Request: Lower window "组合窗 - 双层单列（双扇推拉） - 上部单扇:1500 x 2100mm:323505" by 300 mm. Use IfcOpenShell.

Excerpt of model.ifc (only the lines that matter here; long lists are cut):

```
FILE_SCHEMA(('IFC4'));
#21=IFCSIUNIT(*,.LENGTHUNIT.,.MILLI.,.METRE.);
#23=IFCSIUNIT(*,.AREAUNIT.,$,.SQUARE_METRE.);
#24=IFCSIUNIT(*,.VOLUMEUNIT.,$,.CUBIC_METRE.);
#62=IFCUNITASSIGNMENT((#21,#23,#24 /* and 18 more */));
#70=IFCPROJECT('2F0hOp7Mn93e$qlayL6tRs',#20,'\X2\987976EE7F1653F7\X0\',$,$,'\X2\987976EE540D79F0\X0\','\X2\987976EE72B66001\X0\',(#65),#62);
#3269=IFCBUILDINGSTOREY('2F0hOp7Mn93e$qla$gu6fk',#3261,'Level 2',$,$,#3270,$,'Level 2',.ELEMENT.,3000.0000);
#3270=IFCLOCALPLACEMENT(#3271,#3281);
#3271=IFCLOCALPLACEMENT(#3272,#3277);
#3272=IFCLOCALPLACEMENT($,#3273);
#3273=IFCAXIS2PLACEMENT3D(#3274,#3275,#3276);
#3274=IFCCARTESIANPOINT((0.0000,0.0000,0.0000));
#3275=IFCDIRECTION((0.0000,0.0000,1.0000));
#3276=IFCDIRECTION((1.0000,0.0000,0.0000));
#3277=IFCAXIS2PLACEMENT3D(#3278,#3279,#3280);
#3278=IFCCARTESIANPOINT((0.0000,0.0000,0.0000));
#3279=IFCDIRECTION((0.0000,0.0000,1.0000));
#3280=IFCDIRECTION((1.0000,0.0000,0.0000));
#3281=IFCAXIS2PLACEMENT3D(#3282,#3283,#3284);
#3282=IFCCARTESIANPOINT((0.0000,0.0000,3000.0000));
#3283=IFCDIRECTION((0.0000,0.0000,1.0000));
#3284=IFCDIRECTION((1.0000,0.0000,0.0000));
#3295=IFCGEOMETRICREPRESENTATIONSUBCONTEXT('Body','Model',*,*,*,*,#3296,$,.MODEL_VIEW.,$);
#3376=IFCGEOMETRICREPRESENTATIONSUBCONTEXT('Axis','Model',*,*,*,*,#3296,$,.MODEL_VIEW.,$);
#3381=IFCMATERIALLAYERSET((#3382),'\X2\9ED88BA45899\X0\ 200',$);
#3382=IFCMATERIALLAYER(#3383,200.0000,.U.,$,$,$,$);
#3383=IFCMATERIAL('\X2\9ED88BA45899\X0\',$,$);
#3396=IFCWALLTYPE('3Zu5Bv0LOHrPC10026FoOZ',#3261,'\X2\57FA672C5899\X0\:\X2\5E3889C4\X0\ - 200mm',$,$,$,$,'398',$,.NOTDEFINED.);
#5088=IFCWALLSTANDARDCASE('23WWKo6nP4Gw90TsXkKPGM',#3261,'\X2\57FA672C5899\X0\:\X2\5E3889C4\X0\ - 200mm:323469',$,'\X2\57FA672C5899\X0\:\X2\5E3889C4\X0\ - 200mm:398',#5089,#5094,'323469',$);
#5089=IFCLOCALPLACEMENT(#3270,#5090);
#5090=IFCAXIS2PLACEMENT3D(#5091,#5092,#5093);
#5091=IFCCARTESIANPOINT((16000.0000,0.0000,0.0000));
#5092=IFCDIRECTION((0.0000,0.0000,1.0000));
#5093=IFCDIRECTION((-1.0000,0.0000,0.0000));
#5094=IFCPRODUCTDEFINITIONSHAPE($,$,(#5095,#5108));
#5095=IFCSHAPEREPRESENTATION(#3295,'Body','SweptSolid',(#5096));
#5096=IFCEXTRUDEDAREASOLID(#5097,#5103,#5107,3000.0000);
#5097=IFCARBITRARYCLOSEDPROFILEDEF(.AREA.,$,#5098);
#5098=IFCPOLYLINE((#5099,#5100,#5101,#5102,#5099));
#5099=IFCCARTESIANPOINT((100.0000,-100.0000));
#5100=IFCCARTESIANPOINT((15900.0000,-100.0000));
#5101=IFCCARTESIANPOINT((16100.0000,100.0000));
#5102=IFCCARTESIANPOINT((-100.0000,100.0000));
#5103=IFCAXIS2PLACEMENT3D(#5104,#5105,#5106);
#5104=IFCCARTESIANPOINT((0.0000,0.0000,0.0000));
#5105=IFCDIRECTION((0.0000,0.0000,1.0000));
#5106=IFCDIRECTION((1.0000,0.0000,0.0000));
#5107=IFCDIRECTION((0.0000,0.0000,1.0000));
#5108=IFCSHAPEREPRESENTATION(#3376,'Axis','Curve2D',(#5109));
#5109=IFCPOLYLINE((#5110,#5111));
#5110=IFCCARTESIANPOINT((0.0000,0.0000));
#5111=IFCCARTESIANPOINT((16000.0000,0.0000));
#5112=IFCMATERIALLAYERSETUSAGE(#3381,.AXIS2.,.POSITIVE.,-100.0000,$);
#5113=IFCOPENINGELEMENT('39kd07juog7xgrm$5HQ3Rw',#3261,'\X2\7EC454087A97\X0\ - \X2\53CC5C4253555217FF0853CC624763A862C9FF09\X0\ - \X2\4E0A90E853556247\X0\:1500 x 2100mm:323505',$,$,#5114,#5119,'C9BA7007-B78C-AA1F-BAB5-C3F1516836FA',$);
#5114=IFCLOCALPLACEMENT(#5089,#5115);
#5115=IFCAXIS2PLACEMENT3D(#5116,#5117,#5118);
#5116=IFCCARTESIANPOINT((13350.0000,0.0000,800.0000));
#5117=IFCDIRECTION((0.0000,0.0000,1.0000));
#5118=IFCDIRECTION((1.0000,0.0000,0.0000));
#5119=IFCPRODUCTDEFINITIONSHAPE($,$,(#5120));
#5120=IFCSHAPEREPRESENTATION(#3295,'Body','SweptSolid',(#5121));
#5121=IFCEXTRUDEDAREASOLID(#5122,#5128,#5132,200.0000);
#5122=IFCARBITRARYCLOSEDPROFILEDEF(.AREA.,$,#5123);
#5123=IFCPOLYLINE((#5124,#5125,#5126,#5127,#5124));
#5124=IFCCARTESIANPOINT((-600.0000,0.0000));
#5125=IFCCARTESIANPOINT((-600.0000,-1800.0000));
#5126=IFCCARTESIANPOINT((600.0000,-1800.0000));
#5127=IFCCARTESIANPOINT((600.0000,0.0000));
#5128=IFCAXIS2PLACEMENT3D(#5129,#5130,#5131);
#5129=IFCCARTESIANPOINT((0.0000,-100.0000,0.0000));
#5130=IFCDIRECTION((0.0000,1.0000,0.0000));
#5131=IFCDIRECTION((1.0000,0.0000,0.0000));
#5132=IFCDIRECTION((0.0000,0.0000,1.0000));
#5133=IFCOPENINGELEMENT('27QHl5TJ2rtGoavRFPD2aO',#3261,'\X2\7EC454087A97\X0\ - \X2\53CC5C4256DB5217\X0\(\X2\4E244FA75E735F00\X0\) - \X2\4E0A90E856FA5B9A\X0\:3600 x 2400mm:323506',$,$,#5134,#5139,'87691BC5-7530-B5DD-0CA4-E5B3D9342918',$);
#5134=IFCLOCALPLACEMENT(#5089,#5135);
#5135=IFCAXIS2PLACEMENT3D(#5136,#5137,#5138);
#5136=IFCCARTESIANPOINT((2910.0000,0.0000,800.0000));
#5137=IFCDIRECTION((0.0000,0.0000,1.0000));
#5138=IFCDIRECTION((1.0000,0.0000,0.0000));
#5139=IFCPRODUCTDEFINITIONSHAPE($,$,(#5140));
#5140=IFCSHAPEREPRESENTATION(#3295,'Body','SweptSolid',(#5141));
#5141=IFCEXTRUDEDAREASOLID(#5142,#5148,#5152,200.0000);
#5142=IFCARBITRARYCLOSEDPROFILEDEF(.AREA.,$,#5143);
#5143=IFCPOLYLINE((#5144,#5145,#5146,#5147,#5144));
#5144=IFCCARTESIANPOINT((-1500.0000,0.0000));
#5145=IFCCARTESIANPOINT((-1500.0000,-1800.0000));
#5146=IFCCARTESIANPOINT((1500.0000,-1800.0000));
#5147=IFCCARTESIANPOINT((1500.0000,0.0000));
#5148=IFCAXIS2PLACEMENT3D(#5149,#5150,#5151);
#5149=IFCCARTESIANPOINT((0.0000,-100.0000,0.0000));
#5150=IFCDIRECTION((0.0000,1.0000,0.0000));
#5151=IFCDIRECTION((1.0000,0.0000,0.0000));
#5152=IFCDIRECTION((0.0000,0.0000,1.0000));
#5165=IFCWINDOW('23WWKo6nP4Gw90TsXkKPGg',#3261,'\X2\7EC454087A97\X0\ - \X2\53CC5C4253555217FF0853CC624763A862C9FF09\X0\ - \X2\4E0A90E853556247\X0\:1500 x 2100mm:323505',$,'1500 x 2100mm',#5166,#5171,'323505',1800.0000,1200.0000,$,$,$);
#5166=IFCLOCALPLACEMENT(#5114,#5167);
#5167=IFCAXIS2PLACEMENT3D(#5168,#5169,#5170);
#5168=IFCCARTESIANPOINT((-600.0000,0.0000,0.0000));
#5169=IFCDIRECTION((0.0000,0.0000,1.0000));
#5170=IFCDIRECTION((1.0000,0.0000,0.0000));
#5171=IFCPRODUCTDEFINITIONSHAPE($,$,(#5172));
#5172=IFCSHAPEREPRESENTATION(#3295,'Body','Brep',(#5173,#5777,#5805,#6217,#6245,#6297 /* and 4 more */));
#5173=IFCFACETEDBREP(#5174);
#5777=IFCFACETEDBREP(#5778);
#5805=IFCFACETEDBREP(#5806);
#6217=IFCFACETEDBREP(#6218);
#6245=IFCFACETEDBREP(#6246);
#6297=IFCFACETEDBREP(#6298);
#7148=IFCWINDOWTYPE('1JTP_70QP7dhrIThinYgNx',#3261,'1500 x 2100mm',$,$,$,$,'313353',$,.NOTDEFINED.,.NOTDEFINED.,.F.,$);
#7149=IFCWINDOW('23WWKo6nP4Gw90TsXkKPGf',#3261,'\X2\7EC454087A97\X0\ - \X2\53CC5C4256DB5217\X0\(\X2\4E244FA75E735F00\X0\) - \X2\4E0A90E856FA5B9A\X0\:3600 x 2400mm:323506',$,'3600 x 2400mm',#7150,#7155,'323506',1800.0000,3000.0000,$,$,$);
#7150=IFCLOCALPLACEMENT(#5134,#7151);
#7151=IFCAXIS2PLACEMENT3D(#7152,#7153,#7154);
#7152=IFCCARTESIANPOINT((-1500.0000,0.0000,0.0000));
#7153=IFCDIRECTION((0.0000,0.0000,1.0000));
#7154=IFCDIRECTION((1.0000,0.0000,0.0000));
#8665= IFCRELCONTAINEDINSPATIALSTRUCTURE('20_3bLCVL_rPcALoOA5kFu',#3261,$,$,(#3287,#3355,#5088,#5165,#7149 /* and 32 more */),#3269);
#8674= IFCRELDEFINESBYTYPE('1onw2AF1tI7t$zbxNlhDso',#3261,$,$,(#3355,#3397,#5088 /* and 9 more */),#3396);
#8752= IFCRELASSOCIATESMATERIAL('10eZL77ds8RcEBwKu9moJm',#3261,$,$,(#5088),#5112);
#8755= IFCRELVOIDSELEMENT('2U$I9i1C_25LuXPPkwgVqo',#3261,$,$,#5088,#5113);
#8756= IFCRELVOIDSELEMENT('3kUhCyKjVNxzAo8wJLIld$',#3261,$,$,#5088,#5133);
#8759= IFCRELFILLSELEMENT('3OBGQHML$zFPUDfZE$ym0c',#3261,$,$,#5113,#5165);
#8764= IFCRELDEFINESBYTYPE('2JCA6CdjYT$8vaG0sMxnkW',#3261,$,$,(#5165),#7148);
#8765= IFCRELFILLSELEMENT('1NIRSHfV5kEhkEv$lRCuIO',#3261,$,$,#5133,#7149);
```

```python
import numpy as np
import ifcopenshell
import ifcopenshell.api.geometry
import ifcopenshell.util.placement
import ifcopenshell.util.unit

model = ifcopenshell.open("model.ifc")
unit_scale = ifcopenshell.util.unit.calculate_unit_scale(model)

window = model.by_guid("23WWKo6nP4Gw90TsXkKPGg")
opening = window.FillsVoids[0].RelatingOpeningElement
dz = -0.3 / unit_scale

shift = np.array([0.0, 0.0, dz])
# The window is placed relative to its opening, so it follows when the opening moves.
matrix = ifcopenshell.util.placement.get_local_placement(opening.ObjectPlacement)
matrix[:3, 3] += shift
ifcopenshell.api.geometry.edit_object_placement(
    model, product=opening, matrix=matrix, is_si=False, should_transform_children=True
)

print(f"moved by {dz * unit_scale:+.3f} m")

model.write("model-out.ifc")
```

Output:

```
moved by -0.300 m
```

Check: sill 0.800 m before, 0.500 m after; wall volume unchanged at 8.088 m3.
